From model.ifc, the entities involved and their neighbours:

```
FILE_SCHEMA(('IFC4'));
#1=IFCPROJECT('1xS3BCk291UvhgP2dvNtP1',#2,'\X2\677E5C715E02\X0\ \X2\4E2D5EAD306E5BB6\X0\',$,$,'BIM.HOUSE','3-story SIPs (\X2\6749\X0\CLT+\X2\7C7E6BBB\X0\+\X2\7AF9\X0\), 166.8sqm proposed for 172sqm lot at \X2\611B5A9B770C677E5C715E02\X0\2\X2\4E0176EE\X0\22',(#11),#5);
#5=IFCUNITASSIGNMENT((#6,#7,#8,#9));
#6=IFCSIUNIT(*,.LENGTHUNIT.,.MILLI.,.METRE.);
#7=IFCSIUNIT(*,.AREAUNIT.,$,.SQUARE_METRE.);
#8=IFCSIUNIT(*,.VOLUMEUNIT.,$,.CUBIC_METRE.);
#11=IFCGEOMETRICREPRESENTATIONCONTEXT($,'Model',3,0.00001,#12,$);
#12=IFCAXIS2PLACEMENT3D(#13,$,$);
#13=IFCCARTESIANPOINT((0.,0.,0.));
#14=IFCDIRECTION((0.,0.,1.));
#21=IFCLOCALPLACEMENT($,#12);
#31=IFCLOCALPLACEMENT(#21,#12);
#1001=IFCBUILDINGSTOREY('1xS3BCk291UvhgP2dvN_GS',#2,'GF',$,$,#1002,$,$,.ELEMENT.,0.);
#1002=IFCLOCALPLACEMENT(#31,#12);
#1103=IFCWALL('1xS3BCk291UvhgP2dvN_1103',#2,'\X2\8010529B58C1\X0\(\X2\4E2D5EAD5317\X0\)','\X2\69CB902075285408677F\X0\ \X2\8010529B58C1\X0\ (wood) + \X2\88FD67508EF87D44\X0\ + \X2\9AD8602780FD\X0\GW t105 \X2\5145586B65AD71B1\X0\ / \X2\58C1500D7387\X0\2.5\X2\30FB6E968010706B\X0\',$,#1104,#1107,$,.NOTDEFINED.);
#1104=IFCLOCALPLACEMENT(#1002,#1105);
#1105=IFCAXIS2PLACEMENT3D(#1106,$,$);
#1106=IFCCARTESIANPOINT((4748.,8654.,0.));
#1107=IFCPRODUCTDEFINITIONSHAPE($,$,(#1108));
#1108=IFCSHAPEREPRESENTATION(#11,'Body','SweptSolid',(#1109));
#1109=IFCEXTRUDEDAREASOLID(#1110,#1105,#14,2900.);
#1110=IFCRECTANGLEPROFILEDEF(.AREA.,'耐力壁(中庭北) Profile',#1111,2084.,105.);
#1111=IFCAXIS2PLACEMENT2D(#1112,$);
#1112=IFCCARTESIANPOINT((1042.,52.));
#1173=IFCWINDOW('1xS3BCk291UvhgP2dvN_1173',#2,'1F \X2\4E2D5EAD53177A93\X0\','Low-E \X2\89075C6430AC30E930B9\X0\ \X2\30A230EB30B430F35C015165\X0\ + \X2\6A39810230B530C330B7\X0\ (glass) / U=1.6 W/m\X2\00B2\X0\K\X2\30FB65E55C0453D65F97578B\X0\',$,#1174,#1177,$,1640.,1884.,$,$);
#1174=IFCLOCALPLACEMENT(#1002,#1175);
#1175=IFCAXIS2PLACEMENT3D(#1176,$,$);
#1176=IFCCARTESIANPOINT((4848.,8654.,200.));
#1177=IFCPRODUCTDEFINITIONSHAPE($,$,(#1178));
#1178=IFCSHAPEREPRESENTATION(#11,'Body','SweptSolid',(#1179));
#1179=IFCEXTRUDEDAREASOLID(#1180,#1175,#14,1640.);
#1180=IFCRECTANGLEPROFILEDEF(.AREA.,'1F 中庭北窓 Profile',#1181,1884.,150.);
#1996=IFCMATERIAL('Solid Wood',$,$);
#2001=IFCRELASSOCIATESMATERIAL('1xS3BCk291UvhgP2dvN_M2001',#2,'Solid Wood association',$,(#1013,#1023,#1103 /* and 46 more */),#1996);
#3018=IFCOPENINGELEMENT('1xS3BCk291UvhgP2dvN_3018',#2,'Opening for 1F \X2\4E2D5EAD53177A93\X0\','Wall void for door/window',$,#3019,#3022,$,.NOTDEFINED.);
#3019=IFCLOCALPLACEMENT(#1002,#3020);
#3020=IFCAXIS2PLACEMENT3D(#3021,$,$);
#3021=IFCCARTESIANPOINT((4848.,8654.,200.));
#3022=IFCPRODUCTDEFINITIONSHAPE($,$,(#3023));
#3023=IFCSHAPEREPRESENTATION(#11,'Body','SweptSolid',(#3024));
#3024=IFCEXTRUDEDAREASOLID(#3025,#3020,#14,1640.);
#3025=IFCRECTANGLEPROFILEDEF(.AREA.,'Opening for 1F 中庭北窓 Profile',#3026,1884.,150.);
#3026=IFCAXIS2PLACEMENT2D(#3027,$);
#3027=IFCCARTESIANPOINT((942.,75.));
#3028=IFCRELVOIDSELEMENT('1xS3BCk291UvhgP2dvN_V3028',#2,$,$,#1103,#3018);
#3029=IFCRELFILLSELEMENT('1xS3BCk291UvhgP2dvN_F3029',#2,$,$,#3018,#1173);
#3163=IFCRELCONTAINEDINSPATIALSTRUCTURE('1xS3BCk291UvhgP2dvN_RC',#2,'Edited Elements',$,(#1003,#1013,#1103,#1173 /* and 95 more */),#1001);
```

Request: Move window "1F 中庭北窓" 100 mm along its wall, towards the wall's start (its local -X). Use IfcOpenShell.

```python
import ifcopenshell
import ifcopenshell.api.geometry
import ifcopenshell.util.placement

model = ifcopenshell.open("model.ifc")

window = model.by_guid("1xS3BCk291UvhgP2dvN_1173")
opening = window.FillsVoids[0].RelatingOpeningElement
wall = opening.VoidsElements[0].RelatingBuildingElement

wall_matrix = ifcopenshell.util.placement.get_local_placement(wall.ObjectPlacement)
shift = wall_matrix[:3, 0] * -100.0
before = ifcopenshell.util.placement.get_local_placement(window.ObjectPlacement)[:3, 3].copy()

# The window is not placed relative to its opening, so move both.
for product in (opening, window):
    matrix = ifcopenshell.util.placement.get_local_placement(product.ObjectPlacement)
    matrix[:3, 3] += shift
    ifcopenshell.api.geometry.edit_object_placement(model, product=product, matrix=matrix, is_si=False)

after = ifcopenshell.util.placement.get_local_placement(window.ObjectPlacement)[:3, 3]
print("window moved by", (after - before).round(3) + 0.0)

model.write("model_rev.ifc")
```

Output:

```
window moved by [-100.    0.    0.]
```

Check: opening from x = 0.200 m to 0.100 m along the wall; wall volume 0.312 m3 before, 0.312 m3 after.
